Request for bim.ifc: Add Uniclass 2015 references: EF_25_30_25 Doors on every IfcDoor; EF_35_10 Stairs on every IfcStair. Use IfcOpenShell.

First a look at what the model holds.

```python
import ifcopenshell

model = ifcopenshell.open("bim.ifc")
print(model.schema)
print("classifications:", [c.Name for c in model.by_type("IfcClassification")])
for ifc_class in ("IfcDoor", "IfcRoof", "IfcStair", "IfcWall", "IfcWindow"):
    print(ifc_class, len(model.by_type(ifc_class)))
```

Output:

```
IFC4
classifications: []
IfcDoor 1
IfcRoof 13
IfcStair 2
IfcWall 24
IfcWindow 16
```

```python
import ifcopenshell
import ifcopenshell.api.classification

model = ifcopenshell.open("bim.ifc")

system = ifcopenshell.api.classification.add_classification(model, classification="Uniclass 2015")

codes = {
    "IfcDoor": ("EF_25_30_25", "Doors"),
    "IfcStair": ("EF_35_10", "Stairs"),
}
for ifc_class, (code, name) in codes.items():
    products = model.by_type(ifc_class)
    ifcopenshell.api.classification.add_reference(
        model, products=products, classification=system, identification=code, name=name
    )
    print(code, len(products))

model.write("bim_rev.ifc")
```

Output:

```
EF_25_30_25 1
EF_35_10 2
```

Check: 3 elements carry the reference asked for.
